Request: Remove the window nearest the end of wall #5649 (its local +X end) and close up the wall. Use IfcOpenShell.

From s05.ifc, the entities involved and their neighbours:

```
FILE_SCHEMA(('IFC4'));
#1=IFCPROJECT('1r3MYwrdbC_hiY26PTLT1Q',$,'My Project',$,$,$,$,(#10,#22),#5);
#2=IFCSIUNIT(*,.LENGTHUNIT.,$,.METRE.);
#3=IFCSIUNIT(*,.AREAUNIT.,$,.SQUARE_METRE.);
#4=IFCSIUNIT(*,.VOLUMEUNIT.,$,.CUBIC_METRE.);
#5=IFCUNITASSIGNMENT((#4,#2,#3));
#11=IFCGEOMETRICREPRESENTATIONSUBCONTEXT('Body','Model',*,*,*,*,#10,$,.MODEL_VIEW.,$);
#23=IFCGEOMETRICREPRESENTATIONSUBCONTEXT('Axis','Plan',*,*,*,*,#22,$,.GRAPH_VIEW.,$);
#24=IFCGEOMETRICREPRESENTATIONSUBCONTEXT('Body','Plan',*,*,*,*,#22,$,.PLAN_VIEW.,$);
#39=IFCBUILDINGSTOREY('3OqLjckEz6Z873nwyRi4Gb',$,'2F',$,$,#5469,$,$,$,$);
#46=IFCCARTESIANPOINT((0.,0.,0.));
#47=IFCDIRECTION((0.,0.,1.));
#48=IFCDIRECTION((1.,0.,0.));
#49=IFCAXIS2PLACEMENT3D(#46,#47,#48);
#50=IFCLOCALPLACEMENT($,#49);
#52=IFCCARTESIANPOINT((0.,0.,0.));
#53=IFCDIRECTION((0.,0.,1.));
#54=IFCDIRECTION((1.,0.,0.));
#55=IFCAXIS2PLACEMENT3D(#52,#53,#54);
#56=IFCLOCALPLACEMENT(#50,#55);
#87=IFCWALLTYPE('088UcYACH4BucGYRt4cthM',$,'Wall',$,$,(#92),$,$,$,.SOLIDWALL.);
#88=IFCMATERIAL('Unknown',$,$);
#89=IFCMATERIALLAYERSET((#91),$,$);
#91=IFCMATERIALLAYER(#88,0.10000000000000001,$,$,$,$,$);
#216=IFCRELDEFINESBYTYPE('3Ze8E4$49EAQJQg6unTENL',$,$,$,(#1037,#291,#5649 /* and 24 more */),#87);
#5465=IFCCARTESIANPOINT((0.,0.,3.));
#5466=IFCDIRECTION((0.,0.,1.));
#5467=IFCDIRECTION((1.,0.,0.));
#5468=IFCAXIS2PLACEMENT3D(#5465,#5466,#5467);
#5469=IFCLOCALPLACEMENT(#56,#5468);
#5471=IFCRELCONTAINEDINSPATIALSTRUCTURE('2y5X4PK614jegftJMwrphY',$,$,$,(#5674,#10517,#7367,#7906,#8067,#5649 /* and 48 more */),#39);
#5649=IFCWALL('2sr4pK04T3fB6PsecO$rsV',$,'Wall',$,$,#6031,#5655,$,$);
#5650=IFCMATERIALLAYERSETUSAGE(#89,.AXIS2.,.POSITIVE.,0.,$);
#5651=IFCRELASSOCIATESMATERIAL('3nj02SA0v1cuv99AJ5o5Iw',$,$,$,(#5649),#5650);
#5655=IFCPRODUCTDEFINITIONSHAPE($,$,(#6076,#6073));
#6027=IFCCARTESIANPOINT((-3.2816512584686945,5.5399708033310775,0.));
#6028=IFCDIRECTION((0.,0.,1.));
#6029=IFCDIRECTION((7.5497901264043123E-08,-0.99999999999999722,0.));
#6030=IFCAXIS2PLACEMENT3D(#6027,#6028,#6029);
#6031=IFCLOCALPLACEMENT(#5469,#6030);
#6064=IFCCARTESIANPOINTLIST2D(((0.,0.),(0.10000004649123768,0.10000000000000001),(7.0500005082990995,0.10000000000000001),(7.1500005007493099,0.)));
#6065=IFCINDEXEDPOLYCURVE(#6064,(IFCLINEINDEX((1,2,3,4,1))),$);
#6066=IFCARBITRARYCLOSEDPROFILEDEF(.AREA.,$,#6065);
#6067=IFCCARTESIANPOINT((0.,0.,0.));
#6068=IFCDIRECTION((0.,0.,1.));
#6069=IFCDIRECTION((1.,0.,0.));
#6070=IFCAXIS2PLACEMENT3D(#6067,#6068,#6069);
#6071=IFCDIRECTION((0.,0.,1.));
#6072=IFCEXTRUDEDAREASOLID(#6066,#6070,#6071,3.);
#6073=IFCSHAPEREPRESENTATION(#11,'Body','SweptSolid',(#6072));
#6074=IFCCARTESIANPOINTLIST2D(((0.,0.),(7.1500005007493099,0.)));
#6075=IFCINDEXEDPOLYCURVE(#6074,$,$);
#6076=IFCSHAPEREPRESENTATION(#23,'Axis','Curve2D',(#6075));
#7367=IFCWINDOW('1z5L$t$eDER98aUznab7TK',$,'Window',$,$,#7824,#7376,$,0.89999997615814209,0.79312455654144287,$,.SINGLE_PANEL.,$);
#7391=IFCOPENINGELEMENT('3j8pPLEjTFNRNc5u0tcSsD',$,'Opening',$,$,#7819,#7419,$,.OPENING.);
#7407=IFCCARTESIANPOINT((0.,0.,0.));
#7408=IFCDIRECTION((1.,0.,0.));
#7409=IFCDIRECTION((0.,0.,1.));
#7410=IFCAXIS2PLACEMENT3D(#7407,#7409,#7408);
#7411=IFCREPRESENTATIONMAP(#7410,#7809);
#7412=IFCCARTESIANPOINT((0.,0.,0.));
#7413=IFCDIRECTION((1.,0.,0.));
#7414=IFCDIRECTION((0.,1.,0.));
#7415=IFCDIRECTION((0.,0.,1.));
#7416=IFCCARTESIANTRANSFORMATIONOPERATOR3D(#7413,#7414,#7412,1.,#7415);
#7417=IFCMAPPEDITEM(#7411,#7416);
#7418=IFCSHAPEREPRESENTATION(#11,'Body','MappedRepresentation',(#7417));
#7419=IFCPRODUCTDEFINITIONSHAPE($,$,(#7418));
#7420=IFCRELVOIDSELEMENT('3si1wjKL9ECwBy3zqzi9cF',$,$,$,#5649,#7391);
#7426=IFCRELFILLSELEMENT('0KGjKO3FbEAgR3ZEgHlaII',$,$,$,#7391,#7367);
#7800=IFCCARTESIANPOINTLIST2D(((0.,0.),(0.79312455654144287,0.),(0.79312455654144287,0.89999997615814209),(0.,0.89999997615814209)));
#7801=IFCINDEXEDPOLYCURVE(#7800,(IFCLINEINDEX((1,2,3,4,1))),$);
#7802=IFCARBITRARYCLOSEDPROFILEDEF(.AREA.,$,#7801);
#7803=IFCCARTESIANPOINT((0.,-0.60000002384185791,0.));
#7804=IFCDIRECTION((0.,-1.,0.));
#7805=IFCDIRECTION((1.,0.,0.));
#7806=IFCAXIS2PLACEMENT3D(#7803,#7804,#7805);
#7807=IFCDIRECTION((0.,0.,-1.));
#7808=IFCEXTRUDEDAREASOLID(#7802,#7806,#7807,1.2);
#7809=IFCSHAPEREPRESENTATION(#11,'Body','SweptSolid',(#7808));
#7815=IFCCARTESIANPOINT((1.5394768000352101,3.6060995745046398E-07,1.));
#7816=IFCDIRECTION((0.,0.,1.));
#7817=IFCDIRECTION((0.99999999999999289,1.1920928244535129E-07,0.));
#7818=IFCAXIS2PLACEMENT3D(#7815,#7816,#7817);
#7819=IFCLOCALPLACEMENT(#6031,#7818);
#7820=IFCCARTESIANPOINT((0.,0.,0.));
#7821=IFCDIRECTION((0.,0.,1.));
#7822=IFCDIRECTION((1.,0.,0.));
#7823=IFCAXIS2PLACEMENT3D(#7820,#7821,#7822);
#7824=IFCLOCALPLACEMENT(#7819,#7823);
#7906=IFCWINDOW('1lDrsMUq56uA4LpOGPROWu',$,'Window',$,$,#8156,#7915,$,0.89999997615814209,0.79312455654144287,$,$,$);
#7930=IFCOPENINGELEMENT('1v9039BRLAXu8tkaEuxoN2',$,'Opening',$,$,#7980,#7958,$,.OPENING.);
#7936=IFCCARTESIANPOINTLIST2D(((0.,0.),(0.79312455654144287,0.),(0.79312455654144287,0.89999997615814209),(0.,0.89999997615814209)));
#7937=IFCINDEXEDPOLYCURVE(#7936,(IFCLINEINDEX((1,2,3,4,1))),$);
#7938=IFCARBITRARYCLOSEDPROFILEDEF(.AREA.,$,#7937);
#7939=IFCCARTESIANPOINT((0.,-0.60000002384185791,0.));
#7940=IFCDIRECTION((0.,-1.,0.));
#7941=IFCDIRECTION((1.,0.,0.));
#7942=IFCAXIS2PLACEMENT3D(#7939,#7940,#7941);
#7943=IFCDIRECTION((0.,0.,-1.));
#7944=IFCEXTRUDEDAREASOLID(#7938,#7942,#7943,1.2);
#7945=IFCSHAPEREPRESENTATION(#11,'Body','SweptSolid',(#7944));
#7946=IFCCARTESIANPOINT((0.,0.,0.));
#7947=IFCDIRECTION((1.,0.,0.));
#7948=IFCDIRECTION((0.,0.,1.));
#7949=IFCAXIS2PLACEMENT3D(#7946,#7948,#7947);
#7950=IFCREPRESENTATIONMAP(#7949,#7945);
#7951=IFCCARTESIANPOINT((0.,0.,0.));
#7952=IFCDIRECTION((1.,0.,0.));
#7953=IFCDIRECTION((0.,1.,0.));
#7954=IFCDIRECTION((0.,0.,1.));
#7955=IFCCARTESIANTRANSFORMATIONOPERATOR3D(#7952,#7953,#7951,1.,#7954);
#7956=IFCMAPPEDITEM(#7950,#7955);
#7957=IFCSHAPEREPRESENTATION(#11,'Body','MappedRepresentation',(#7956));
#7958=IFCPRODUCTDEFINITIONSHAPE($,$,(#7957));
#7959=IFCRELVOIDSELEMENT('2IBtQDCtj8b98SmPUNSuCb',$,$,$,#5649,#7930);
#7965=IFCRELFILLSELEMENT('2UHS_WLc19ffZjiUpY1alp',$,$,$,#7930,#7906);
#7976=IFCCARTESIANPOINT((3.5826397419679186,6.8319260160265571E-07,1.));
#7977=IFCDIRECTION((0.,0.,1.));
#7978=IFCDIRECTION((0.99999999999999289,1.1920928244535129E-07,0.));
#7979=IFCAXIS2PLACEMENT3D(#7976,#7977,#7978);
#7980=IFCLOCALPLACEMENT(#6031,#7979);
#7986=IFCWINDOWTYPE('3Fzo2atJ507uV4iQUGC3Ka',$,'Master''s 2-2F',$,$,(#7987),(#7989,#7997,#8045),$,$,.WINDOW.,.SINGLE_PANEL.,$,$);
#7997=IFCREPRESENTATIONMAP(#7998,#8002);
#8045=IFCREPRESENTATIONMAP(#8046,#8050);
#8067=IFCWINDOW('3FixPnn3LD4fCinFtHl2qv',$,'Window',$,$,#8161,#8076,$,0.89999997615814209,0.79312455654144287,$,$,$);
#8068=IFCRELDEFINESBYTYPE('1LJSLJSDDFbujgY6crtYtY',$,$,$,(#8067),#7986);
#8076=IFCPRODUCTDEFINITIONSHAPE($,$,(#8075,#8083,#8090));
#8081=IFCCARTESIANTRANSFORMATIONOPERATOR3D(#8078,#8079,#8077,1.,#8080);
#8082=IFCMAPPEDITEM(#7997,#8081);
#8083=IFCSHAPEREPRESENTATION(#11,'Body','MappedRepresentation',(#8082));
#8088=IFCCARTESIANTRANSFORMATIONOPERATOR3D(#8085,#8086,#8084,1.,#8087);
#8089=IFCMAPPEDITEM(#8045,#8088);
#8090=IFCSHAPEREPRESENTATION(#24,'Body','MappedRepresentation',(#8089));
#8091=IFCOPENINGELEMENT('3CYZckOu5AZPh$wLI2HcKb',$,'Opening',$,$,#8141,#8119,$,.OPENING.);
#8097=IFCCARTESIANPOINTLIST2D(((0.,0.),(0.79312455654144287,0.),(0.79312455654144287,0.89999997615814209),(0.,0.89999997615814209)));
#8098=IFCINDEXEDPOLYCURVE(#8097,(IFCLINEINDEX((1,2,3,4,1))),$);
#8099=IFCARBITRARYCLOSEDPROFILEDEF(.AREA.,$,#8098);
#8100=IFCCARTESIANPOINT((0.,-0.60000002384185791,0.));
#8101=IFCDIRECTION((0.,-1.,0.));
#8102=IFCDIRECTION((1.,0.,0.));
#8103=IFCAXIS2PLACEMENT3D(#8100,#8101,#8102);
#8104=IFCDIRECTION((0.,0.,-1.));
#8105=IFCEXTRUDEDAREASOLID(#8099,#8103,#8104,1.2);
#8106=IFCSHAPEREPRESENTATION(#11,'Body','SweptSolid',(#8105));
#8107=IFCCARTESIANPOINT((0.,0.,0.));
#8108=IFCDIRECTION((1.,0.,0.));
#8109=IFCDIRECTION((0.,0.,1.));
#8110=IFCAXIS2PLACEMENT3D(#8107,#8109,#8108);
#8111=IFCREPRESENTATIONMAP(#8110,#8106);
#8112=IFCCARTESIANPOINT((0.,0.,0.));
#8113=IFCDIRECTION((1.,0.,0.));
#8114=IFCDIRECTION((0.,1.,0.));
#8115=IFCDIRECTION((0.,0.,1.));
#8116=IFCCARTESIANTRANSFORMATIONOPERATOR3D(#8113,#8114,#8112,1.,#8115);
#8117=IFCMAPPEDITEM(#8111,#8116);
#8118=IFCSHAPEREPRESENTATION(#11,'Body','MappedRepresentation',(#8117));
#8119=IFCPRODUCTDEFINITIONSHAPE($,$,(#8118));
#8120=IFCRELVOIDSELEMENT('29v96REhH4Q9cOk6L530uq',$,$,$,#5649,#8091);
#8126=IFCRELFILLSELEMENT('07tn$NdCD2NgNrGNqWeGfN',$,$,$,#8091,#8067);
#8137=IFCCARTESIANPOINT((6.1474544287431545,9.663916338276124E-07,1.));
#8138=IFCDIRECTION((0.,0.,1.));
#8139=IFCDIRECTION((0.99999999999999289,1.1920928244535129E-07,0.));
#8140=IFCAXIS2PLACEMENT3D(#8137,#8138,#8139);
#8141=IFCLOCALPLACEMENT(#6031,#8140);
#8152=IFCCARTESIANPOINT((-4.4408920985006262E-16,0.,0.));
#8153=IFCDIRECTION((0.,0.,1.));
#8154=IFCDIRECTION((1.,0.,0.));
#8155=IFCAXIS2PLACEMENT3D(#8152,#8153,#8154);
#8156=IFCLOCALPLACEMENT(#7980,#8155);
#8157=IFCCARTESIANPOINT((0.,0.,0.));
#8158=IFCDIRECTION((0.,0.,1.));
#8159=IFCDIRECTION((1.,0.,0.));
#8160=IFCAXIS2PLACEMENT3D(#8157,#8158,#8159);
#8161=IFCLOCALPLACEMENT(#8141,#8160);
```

```python
import ifcopenshell
import ifcopenshell.api.feature
import ifcopenshell.api.root
import ifcopenshell.geom
import ifcopenshell.util.shape

model = ifcopenshell.open("s05.ifc")
settings = ifcopenshell.geom.settings()


def volume(element):
    """Net volume in cubic metres, openings subtracted."""
    shape = ifcopenshell.geom.create_shape(settings, element)
    return ifcopenshell.util.shape.get_volume(shape.geometry)


window = model.by_guid("3FixPnn3LD4fCinFtHl2qv")
opening = window.FillsVoids[0].RelatingOpeningElement
wall = opening.VoidsElements[0].RelatingBuildingElement
before = volume(wall)

ifcopenshell.api.root.remove_product(model, product=window)
ifcopenshell.api.feature.remove_feature(model, feature=opening)

after = volume(wall)

print(f"wall volume {before:.3f} -> {after:.3f} m3")

model.write("s05_v2.ifc")
```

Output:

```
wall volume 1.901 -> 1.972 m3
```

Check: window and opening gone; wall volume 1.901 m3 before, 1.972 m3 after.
